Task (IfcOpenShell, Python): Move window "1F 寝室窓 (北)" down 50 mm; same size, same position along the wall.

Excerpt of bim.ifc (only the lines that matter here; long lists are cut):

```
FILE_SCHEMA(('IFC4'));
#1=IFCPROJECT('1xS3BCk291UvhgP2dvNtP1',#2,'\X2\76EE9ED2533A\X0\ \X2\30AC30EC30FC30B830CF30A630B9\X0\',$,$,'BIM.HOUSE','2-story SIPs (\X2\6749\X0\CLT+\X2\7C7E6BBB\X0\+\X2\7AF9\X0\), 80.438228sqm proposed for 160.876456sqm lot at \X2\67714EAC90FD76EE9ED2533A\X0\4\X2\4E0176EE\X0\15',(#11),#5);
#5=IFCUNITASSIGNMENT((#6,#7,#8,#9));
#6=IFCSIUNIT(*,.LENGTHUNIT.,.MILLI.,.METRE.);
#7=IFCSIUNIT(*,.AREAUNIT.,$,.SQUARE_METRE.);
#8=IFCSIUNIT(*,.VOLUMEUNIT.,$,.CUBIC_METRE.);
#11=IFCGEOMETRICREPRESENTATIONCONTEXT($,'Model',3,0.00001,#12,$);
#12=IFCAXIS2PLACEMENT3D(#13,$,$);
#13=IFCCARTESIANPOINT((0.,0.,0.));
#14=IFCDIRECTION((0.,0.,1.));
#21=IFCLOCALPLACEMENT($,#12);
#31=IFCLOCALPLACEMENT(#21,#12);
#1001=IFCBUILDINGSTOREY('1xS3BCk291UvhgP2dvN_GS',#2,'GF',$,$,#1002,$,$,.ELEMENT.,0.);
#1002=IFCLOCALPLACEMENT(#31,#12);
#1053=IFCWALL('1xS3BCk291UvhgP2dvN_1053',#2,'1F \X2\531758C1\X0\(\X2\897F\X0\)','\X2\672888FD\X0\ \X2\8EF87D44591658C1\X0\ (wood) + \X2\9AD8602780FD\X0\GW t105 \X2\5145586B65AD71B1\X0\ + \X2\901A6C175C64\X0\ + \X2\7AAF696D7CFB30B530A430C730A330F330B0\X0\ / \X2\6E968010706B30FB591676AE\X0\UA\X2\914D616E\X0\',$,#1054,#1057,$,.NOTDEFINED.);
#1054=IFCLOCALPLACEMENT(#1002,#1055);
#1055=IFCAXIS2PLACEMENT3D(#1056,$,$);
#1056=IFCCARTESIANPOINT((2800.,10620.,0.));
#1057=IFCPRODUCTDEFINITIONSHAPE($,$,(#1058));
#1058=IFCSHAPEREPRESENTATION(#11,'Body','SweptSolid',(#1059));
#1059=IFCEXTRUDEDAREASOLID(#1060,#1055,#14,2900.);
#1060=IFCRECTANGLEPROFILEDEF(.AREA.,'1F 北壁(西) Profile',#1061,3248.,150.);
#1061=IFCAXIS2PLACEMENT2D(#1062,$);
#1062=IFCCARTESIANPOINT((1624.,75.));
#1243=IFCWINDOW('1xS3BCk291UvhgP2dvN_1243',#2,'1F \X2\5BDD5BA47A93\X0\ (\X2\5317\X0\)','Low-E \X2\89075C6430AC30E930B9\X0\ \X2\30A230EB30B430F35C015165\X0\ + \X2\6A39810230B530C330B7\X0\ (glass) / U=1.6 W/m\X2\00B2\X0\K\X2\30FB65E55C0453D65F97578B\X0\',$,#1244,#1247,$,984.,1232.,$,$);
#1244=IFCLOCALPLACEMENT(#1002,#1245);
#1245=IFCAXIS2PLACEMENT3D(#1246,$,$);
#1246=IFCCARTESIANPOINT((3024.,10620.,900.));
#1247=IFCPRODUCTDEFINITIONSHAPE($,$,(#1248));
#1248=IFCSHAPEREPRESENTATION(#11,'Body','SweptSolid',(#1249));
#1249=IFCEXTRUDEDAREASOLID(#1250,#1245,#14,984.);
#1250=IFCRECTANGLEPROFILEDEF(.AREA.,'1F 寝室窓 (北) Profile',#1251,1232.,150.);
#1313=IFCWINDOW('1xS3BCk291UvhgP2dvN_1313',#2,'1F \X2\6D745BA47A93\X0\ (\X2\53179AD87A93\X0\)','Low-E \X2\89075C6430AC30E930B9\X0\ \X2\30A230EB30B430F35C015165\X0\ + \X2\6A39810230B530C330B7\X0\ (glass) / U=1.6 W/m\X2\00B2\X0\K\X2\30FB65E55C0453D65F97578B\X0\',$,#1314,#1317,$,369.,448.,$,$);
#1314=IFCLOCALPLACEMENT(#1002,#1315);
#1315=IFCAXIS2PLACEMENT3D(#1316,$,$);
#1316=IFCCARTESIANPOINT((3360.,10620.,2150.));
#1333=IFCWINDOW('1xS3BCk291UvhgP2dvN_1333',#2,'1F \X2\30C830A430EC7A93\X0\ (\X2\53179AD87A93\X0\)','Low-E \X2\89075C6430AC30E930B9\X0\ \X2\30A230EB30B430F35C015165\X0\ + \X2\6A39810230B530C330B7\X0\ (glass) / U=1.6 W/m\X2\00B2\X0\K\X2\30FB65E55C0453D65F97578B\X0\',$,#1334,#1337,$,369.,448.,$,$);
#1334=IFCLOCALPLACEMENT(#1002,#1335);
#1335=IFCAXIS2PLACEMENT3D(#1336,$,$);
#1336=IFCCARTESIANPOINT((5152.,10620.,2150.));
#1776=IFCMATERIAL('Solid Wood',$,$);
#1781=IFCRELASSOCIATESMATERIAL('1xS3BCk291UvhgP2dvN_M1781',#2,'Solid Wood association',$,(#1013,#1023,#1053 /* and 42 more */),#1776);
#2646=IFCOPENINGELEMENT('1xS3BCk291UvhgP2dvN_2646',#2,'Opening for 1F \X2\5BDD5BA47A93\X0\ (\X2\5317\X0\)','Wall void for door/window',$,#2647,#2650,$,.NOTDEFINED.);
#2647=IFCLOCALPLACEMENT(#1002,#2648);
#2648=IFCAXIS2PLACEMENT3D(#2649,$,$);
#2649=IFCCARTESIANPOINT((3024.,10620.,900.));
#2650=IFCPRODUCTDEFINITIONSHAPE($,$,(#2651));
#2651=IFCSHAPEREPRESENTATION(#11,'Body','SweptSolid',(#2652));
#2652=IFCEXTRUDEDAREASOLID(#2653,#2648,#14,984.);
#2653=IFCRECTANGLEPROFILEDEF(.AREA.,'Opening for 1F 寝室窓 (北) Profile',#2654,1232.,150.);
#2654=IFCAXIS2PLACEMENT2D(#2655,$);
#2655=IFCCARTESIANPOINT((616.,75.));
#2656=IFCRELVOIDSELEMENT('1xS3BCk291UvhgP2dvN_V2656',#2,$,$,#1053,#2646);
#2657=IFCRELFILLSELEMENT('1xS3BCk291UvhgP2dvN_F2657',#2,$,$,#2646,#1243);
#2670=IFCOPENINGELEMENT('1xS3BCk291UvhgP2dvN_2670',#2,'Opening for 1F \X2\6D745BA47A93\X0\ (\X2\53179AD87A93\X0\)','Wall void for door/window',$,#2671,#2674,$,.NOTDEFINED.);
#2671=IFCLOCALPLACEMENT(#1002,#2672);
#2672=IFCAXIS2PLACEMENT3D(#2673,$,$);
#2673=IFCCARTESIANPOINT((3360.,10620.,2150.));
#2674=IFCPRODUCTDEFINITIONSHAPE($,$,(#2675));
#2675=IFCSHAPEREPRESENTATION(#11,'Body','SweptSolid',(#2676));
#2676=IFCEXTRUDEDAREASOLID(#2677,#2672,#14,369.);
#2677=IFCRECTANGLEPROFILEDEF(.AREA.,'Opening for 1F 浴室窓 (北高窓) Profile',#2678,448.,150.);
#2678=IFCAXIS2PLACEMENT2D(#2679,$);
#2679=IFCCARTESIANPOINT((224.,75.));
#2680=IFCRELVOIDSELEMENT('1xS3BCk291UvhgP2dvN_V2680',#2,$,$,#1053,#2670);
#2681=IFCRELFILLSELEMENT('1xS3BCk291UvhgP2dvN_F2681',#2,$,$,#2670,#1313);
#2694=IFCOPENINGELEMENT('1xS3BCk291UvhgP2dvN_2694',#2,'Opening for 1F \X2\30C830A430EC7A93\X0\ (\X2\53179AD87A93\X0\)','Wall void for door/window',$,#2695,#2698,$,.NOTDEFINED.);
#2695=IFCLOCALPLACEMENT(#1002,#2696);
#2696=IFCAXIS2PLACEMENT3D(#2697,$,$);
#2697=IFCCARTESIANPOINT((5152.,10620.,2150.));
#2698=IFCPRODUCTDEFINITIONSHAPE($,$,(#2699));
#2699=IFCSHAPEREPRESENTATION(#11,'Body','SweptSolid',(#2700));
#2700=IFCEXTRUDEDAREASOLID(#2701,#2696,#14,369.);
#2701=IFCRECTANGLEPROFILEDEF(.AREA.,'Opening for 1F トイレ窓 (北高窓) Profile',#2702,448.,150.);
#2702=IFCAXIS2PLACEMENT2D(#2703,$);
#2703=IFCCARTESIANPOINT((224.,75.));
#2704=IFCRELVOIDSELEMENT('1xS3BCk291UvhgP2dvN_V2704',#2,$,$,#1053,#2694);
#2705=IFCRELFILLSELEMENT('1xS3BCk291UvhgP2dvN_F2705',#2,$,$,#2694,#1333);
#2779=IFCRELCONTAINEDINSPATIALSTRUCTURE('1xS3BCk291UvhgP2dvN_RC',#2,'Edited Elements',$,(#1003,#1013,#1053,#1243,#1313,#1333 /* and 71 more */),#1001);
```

```python
import numpy as np
import ifcopenshell
import ifcopenshell.api.geometry
import ifcopenshell.util.placement
import ifcopenshell.util.unit

model = ifcopenshell.open("bim.ifc")
unit_scale = ifcopenshell.util.unit.calculate_unit_scale(model)

window = model.by_guid("1xS3BCk291UvhgP2dvN_1243")
opening = window.FillsVoids[0].RelatingOpeningElement
dz = -50.0

shift = np.array([0.0, 0.0, dz])
# The window is not placed relative to its opening, so move both.
for product in (opening, window):
    matrix = ifcopenshell.util.placement.get_local_placement(product.ObjectPlacement)
    matrix[:3, 3] += shift
    ifcopenshell.api.geometry.edit_object_placement(model, product=product, matrix=matrix, is_si=False)

print(f"moved by {dz * unit_scale:+.3f} m")

model.write("bim-out.ifc")
```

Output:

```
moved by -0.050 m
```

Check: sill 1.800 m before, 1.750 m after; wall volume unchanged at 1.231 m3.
